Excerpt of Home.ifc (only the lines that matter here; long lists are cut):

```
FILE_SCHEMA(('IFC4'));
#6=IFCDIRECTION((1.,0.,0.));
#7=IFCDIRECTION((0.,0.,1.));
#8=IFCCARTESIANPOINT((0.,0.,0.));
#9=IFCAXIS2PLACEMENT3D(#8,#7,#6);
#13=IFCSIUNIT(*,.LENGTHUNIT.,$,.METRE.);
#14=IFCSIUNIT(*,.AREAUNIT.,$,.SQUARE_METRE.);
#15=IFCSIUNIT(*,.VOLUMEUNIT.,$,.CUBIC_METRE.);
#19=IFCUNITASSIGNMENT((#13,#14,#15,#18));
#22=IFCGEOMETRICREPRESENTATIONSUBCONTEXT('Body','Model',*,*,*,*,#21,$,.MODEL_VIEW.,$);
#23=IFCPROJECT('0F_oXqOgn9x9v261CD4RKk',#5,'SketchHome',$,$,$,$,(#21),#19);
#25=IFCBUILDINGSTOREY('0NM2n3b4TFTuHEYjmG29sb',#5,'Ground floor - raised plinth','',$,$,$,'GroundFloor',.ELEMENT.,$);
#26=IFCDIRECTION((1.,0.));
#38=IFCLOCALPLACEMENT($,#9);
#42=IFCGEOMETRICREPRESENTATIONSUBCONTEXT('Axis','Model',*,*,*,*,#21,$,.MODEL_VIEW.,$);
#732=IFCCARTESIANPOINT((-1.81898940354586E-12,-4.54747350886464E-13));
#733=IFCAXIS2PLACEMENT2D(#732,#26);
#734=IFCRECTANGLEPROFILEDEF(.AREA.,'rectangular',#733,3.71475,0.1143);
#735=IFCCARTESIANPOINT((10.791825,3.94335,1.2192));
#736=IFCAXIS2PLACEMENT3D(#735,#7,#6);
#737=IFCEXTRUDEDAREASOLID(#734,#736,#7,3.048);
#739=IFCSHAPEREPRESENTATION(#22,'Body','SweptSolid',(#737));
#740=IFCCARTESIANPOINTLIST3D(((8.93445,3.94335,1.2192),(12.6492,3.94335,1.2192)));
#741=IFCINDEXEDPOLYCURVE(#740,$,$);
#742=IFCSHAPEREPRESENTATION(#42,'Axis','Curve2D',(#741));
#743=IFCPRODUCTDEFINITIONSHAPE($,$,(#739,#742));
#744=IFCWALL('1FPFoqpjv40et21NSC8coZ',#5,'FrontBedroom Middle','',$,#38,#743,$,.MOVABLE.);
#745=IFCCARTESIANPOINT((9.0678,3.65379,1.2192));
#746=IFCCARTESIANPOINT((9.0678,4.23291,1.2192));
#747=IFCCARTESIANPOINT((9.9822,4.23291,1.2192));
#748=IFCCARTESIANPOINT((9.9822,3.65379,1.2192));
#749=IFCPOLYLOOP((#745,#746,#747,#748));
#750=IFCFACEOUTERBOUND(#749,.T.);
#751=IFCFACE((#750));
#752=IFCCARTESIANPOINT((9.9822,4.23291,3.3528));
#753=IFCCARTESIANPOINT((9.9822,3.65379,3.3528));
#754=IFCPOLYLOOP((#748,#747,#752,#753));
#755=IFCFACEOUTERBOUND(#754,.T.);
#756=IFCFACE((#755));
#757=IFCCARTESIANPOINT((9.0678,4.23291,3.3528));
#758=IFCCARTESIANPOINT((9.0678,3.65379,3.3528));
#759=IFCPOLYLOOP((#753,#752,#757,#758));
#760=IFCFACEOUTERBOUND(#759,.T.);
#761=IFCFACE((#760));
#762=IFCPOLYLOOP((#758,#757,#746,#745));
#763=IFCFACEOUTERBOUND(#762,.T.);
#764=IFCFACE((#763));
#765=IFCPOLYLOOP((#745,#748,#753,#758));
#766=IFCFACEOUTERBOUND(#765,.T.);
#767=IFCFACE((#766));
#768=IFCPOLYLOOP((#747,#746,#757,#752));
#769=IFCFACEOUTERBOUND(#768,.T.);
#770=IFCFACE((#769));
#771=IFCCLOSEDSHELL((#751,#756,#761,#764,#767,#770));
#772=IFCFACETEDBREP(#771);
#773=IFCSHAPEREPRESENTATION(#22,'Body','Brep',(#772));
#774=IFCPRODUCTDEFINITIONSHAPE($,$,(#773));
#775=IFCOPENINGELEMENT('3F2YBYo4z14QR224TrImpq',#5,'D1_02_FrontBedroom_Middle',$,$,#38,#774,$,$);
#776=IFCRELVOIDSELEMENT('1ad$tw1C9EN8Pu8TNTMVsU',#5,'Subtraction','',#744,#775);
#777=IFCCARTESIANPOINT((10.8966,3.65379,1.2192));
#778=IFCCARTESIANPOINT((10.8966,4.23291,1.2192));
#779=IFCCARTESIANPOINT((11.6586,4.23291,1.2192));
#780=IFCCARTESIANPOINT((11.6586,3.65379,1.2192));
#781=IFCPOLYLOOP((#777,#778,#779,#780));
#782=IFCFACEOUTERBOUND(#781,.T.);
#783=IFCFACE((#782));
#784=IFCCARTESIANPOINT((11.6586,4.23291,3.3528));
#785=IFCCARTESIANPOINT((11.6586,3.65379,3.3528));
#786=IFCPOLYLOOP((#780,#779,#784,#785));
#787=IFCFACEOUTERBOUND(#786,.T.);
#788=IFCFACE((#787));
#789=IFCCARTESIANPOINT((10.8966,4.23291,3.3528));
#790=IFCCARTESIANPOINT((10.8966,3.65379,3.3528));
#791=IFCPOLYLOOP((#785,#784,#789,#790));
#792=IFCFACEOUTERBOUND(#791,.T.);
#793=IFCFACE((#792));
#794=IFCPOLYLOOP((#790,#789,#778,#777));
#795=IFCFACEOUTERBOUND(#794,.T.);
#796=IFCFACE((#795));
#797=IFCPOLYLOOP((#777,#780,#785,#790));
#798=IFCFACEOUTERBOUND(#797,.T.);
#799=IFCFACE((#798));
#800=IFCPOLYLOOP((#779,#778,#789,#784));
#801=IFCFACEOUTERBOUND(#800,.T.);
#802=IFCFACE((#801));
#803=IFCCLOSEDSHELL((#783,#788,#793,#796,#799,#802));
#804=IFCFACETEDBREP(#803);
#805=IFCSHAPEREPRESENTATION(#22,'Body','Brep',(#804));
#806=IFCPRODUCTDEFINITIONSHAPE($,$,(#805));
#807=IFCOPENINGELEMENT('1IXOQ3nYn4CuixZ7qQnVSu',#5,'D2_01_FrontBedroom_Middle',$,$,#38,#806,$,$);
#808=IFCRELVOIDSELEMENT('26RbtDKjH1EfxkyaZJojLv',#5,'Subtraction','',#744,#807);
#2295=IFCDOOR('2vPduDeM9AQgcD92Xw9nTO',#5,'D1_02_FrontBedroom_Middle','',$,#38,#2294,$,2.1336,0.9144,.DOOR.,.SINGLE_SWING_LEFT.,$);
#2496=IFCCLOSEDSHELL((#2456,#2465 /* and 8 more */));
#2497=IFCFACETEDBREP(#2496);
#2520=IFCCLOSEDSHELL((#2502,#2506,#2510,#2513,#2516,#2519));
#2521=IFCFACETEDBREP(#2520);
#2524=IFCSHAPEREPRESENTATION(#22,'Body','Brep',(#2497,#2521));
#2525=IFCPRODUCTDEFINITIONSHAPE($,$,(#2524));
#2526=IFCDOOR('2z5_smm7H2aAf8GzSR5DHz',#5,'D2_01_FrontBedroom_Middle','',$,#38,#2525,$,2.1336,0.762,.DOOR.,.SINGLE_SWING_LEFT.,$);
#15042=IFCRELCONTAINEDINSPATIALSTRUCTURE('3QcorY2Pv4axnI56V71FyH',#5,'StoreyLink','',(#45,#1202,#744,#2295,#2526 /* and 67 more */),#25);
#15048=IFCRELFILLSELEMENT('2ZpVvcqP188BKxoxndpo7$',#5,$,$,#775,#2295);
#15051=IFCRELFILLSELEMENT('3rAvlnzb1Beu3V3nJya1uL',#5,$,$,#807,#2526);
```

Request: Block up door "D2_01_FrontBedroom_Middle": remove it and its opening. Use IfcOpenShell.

```python
import ifcopenshell
import ifcopenshell.api.feature
import ifcopenshell.api.root
import ifcopenshell.geom
import ifcopenshell.util.shape

model = ifcopenshell.open("Home.ifc")
settings = ifcopenshell.geom.settings()


def volume(element):
    """Net volume in cubic metres, openings subtracted."""
    shape = ifcopenshell.geom.create_shape(settings, element)
    return ifcopenshell.util.shape.get_volume(shape.geometry)


door = model.by_guid("2z5_smm7H2aAf8GzSR5DHz")
opening = door.FillsVoids[0].RelatingOpeningElement
wall = opening.VoidsElements[0].RelatingBuildingElement
before = volume(wall)

ifcopenshell.api.root.remove_product(model, product=door)
ifcopenshell.api.feature.remove_feature(model, feature=opening)

after = volume(wall)

print(f"wall volume {before:.3f} -> {after:.3f} m3")

model.write("Home-out.ifc")
```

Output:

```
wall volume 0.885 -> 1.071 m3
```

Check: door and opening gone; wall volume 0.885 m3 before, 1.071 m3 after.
